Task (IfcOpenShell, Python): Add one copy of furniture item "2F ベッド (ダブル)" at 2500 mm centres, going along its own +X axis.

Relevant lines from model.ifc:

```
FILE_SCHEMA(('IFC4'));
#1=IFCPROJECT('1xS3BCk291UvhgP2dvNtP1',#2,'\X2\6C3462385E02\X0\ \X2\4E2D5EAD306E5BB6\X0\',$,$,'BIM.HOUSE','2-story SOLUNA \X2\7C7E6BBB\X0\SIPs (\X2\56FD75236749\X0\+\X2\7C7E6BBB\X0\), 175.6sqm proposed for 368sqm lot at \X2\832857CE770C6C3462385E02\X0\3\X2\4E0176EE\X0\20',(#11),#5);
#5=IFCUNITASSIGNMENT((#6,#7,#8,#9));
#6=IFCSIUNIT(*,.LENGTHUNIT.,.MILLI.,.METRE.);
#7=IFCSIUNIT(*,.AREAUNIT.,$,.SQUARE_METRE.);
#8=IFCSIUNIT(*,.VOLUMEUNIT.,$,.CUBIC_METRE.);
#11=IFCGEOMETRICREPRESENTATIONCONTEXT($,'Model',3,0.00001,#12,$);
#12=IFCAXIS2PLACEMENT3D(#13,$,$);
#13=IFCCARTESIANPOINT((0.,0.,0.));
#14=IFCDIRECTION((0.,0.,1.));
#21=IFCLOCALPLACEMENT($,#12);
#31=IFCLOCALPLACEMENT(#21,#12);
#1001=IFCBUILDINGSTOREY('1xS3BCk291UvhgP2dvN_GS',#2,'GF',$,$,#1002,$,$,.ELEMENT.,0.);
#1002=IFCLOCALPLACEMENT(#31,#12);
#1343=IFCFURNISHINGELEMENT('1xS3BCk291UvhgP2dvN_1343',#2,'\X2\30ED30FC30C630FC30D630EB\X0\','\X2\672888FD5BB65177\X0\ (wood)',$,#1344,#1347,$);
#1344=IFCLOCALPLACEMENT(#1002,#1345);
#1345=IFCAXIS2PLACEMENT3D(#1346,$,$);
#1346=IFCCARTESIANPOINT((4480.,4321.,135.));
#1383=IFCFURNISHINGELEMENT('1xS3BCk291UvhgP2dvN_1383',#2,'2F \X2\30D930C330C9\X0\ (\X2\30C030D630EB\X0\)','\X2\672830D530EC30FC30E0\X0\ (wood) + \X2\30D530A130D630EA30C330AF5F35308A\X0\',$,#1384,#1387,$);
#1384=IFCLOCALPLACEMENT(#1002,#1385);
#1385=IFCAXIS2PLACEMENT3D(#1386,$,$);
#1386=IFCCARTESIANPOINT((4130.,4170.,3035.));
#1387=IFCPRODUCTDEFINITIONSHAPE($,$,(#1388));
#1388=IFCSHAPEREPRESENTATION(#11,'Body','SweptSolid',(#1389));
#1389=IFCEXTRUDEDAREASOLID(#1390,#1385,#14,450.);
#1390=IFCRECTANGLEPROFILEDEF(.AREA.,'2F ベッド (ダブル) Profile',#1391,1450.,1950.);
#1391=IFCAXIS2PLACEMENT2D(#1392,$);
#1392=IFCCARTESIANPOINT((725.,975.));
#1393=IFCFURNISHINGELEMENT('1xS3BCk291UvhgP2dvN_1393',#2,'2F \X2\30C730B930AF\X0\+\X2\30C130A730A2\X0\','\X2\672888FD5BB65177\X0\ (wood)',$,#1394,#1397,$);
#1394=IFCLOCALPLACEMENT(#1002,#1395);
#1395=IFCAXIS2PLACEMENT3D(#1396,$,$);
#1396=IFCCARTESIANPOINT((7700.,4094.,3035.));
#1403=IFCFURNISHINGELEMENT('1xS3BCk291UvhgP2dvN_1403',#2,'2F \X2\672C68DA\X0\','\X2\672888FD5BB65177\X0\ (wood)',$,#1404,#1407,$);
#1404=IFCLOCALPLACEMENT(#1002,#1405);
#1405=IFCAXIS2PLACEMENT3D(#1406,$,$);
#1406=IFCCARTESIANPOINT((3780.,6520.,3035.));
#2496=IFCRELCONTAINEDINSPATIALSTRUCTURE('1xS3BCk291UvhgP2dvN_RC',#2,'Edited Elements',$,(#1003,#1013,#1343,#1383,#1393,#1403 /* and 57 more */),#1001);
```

```python
import ifcopenshell
import ifcopenshell.api.geometry
import ifcopenshell.api.root
import ifcopenshell.util.element
import ifcopenshell.util.placement
import ifcopenshell.util.unit

model = ifcopenshell.open("model.ifc")
unit_scale = ifcopenshell.util.unit.calculate_unit_scale(model)


def reuse_history(source, copy):
    """copy_class also copies each property set's owner history, people and application; keep the originals."""
    for rel in copy.IsDefinedBy:
        if rel.is_a("IfcRelDefinesByProperties") and (history := rel.RelatingPropertyDefinition.OwnerHistory):
            rel.RelatingPropertyDefinition.OwnerHistory = source.OwnerHistory
            ifcopenshell.util.element.remove_deep2(model, history)


source = model.by_guid("1xS3BCk291UvhgP2dvN_1383")
base = ifcopenshell.util.placement.get_local_placement(source.ObjectPlacement)
step = base[:3, 0] * 2.5 / unit_scale

for i in range(1, 2):
    copy = ifcopenshell.api.root.copy_class(model, product=source)
    copy.Representation = ifcopenshell.util.element.copy_deep(
        model, source.Representation, exclude=["IfcGeometricRepresentationContext", "IfcRepresentationMap"]
    )
    reuse_history(source, copy)
    matrix = base.copy()
    matrix[:3, 3] += i * step
    print("added at", matrix[:3, 3].round(3) + 0.0)
    ifcopenshell.api.geometry.edit_object_placement(model, product=copy, matrix=matrix, is_si=False)

model.write("model_edited.ifc")
```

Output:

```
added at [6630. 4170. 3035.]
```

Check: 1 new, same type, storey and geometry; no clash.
